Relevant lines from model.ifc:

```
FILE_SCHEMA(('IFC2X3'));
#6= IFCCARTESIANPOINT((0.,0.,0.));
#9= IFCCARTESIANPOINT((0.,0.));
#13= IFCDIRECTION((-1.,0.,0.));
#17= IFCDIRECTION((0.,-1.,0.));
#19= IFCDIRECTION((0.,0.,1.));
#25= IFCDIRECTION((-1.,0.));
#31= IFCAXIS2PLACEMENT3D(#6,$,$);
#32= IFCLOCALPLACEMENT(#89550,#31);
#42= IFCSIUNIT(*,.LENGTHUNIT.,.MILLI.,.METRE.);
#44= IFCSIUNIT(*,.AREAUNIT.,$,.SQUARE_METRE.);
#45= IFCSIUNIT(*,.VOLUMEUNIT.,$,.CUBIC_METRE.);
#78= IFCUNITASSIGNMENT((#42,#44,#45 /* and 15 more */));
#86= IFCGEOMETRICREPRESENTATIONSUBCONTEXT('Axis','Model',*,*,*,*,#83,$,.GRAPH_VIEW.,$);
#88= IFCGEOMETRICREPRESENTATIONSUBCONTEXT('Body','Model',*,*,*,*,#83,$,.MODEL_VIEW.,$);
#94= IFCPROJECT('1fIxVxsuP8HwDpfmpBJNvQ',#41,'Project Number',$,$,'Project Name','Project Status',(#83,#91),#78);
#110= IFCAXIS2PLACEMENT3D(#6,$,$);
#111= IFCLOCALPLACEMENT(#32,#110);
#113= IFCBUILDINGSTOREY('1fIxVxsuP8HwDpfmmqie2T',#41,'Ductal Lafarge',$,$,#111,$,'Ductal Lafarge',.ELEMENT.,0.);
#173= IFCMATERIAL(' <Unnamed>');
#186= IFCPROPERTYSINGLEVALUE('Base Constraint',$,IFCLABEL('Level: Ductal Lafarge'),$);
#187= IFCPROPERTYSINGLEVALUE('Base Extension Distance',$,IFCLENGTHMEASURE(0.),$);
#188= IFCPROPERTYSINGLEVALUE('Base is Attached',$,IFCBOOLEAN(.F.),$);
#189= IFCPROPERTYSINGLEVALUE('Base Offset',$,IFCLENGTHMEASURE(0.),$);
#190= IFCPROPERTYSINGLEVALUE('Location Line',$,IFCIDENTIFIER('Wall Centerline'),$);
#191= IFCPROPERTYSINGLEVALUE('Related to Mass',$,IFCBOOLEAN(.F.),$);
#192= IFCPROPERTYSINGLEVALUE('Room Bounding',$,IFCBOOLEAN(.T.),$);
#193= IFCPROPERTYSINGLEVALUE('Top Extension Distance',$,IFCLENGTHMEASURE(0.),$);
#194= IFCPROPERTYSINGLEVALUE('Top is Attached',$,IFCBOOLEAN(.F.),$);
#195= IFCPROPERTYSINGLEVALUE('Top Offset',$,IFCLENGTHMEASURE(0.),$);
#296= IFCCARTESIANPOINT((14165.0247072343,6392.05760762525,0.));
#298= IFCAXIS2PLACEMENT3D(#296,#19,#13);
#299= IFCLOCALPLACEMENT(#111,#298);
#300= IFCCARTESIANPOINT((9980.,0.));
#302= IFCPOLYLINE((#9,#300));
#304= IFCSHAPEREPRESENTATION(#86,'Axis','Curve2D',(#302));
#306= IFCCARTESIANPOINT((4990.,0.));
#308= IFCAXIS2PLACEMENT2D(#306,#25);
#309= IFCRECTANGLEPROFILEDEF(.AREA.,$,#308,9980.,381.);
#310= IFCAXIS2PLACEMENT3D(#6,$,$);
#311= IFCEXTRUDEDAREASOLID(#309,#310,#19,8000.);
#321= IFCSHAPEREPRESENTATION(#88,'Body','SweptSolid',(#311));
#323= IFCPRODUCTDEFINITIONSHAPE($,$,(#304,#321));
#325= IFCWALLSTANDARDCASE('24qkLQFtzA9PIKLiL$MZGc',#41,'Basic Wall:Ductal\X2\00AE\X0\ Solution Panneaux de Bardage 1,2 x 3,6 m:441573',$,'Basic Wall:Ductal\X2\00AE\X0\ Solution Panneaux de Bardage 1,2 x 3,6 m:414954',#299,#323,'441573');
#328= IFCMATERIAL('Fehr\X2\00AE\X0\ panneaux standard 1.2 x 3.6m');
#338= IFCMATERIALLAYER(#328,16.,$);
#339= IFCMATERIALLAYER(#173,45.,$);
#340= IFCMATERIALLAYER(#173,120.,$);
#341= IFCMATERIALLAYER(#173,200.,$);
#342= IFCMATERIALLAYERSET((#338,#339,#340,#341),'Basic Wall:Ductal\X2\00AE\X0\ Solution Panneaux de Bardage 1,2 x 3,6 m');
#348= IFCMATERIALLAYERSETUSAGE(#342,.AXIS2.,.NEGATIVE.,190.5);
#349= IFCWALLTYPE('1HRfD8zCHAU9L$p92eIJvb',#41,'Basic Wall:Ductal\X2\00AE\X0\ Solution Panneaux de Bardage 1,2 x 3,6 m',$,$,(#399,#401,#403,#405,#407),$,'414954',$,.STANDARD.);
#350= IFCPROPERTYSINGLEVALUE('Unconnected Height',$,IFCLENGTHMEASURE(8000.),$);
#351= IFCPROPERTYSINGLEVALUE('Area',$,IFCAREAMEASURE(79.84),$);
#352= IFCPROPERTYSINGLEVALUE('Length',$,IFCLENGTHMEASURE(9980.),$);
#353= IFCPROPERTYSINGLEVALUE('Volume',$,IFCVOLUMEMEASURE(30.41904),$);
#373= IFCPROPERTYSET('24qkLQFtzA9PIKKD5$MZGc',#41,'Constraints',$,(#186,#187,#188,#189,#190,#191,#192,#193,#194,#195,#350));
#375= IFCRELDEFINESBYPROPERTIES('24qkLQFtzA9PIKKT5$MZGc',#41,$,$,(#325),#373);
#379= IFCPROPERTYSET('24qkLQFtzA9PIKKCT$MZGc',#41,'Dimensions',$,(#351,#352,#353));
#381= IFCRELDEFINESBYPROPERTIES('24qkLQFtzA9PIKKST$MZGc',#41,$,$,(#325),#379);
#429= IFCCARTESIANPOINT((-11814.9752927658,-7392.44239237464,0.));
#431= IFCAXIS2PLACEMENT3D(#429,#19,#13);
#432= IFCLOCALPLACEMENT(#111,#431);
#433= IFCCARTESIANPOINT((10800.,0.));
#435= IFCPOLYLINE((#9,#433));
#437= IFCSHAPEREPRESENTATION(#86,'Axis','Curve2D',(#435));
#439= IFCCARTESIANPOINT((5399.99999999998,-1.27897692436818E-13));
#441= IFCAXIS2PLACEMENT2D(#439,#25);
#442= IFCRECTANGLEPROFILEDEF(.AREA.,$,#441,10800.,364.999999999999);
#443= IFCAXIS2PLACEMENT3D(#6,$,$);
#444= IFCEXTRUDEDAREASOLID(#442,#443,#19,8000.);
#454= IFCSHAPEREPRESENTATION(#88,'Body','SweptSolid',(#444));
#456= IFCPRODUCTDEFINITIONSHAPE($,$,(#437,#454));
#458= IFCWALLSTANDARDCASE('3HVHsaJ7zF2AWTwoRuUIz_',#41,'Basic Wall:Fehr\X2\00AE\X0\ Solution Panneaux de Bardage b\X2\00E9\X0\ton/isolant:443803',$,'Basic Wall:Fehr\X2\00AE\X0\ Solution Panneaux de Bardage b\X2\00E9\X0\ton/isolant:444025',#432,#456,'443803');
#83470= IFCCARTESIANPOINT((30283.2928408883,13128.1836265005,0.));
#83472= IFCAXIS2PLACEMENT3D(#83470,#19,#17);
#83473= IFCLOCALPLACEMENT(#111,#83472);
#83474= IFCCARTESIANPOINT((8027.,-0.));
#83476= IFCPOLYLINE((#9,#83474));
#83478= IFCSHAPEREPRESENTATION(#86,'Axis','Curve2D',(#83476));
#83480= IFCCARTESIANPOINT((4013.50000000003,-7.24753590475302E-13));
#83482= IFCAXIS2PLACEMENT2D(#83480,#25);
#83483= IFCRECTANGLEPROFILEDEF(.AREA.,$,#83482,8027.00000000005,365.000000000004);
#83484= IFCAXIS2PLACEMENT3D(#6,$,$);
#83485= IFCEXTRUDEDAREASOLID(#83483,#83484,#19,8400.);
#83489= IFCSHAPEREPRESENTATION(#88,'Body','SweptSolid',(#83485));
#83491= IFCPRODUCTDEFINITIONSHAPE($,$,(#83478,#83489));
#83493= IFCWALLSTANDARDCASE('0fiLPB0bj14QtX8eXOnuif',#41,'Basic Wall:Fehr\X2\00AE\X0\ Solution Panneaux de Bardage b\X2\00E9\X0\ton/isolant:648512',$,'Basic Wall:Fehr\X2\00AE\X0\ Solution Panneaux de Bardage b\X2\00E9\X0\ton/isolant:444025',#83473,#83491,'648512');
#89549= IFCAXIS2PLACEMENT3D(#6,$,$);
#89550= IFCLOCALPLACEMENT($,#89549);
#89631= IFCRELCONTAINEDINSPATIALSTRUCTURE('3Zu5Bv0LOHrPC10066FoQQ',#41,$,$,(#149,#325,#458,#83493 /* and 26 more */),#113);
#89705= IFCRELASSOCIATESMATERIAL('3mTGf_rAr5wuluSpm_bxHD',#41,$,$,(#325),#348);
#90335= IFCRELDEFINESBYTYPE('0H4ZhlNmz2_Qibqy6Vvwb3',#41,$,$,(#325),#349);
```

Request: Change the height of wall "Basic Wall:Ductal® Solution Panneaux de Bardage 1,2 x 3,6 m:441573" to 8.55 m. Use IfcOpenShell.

```python
import ifcopenshell
import ifcopenshell.api.pset
import ifcopenshell.geom
import ifcopenshell.util.element
import ifcopenshell.util.representation
import ifcopenshell.util.shape
import ifcopenshell.util.unit

model = ifcopenshell.open("model.ifc")
unit_scale = ifcopenshell.util.unit.calculate_unit_scale(model)
area_scale = ifcopenshell.util.unit.calculate_unit_scale(model, "AREAUNIT")
volume_scale = ifcopenshell.util.unit.calculate_unit_scale(model, "VOLUMEUNIT")
settings = ifcopenshell.geom.settings()


def volume(element):
    """Net volume in cubic metres, openings subtracted."""
    shape = ifcopenshell.geom.create_shape(settings, element)
    return ifcopenshell.util.shape.get_volume(shape.geometry)


wall = model.by_guid("24qkLQFtzA9PIKLiL$MZGc")
before = volume(wall)

body = ifcopenshell.util.representation.get_representation(wall, "Model", "Body")
solid = body.Items[0]
old_height = solid.Depth
solid.Depth = 8.55 / unit_scale
after = volume(wall)
thickness = 0.381  # wall thickness in metres

# Update the stored height, areas and volumes.
pset = model.by_id(ifcopenshell.util.element.get_pset(wall, "Constraints", should_inherit=False)["id"])
ifcopenshell.api.pset.edit_pset(model, pset=pset, properties={
    "Unconnected Height": model.create_entity("IfcLengthMeasure", solid.Depth),
})
pset = model.by_id(ifcopenshell.util.element.get_pset(wall, "Dimensions", should_inherit=False)["id"])
ifcopenshell.api.pset.edit_pset(model, pset=pset, properties={
    "Area": model.create_entity("IfcAreaMeasure", after / thickness / area_scale),
    "Volume": model.create_entity("IfcVolumeMeasure", after / volume_scale),
})

print(f"height {old_height:g} -> {solid.Depth:g}, volume {before:.3f} -> {after:.3f} m3")

model.write("model_rev.ifc")
```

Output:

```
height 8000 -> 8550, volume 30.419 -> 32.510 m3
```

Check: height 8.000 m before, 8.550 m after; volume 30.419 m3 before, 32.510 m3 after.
